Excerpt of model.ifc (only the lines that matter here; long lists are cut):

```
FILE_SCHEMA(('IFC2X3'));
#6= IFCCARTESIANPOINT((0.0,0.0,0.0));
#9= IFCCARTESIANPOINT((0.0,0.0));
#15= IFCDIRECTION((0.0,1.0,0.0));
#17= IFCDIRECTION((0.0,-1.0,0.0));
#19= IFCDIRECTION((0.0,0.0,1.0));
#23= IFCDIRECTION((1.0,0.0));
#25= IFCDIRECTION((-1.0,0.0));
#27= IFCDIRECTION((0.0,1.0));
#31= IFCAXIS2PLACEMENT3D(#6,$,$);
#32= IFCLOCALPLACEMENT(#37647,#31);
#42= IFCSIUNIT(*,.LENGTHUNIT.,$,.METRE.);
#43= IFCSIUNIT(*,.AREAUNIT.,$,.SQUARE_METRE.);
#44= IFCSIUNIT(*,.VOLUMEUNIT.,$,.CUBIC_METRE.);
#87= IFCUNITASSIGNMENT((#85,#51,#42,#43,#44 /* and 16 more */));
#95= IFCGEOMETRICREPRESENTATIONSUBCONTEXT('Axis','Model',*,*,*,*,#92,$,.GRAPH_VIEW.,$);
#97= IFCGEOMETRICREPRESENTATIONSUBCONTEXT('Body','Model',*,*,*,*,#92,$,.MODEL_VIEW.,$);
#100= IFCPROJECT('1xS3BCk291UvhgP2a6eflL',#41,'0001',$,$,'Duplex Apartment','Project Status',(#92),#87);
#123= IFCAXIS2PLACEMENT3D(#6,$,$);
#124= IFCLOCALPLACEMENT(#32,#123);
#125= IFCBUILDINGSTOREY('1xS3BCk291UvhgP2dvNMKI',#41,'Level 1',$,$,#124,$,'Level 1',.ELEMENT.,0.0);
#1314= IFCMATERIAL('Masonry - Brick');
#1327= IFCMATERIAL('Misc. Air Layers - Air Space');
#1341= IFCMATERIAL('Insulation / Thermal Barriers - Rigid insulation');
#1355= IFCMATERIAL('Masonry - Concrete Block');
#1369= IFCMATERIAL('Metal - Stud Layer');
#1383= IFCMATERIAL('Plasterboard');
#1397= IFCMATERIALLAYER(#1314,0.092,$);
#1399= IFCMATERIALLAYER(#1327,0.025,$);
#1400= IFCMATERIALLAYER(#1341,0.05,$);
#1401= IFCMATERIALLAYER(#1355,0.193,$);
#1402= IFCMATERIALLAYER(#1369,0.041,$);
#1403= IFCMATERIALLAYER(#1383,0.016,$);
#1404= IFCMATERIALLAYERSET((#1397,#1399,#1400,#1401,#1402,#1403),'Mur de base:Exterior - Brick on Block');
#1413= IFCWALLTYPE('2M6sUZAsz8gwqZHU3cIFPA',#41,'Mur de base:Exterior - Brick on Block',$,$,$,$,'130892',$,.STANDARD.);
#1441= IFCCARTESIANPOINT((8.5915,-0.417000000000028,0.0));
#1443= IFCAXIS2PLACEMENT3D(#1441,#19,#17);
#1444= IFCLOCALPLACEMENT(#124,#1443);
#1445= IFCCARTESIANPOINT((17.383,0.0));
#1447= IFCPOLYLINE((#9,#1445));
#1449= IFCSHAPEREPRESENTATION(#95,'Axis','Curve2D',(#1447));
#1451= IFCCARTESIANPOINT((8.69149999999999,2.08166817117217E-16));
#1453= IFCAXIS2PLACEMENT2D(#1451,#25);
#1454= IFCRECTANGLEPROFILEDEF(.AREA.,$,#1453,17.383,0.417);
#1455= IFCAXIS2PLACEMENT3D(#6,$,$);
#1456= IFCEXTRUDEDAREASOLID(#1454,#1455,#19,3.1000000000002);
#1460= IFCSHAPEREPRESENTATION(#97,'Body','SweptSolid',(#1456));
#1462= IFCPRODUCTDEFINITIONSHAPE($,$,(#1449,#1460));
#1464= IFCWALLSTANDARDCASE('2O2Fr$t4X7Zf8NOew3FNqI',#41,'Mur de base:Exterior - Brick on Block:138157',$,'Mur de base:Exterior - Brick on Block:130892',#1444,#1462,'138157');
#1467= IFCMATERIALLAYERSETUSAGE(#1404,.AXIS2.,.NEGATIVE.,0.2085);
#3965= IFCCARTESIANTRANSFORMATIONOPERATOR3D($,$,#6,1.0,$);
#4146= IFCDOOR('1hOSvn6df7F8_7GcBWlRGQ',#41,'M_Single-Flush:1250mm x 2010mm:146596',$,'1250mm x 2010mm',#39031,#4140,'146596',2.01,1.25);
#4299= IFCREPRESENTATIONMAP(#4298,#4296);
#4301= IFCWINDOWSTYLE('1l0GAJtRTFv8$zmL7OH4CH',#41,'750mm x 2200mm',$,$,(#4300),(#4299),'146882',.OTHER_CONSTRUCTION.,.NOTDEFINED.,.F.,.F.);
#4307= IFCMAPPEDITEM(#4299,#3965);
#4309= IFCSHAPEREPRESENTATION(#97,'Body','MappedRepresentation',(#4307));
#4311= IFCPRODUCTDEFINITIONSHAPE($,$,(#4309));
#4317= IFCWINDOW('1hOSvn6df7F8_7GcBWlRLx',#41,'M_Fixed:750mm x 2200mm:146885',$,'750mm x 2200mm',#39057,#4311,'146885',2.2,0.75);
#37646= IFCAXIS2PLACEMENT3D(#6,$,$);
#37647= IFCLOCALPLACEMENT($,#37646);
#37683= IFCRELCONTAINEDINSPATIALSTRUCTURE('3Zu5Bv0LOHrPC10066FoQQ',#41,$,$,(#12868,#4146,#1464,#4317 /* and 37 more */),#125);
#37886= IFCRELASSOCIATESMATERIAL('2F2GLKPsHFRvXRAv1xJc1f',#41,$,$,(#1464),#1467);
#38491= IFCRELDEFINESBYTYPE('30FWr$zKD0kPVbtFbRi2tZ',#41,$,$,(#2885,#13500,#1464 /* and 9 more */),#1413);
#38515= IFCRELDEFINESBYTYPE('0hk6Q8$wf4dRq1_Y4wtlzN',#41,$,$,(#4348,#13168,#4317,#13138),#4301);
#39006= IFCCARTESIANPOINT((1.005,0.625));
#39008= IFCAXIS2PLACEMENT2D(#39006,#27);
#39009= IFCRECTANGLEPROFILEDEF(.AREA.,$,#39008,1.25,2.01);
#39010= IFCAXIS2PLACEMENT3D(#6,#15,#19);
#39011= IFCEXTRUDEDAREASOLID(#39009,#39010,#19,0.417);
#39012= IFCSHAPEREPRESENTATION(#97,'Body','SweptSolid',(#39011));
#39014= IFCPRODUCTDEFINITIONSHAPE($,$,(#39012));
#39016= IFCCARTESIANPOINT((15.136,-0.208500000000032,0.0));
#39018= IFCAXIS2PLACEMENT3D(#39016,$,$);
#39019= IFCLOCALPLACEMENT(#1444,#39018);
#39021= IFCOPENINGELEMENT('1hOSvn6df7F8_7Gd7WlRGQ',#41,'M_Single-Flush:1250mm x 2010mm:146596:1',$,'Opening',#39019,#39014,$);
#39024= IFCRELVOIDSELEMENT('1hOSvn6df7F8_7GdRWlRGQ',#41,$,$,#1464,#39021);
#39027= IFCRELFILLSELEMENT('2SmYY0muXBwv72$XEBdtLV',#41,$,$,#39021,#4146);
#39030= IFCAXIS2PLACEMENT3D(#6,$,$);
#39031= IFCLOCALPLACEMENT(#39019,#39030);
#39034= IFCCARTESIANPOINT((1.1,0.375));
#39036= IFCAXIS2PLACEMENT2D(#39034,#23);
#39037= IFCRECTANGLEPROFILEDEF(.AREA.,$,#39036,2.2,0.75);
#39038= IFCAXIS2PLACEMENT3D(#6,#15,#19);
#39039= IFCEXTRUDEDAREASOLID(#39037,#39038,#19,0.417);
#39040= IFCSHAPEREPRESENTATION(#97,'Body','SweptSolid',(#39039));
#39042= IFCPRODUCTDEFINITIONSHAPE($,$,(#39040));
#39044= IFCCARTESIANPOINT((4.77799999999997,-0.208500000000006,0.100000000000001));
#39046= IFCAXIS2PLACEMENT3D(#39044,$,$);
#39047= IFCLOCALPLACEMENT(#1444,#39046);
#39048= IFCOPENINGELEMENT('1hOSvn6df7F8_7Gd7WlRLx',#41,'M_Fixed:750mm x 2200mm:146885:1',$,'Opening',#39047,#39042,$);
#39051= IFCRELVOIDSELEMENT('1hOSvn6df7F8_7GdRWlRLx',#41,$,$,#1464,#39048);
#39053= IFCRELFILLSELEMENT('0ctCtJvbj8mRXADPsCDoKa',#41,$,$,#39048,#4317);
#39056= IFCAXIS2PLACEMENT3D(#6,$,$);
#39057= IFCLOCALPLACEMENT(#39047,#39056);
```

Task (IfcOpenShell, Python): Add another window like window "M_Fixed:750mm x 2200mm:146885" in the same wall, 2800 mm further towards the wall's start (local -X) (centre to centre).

```python
import ifcopenshell
import ifcopenshell.api.feature
import ifcopenshell.api.geometry
import ifcopenshell.api.root
import ifcopenshell.geom
import ifcopenshell.util.element
import ifcopenshell.util.placement
import ifcopenshell.util.shape
import ifcopenshell.util.unit

model = ifcopenshell.open("model.ifc")
unit_scale = ifcopenshell.util.unit.calculate_unit_scale(model)
settings = ifcopenshell.geom.settings()


def volume(element):
    """Net volume in cubic metres, openings subtracted."""
    shape = ifcopenshell.geom.create_shape(settings, element)
    return ifcopenshell.util.shape.get_volume(shape.geometry)


def reuse_history(source, copy):
    """copy_class also copies each property set's owner history, people and application; keep the originals."""
    for rel in copy.IsDefinedBy:
        if rel.is_a("IfcRelDefinesByProperties") and (history := rel.RelatingPropertyDefinition.OwnerHistory):
            rel.RelatingPropertyDefinition.OwnerHistory = source.OwnerHistory
            ifcopenshell.util.element.remove_deep2(model, history)


window = model.by_guid("1hOSvn6df7F8_7GcBWlRLx")
opening = window.FillsVoids[0].RelatingOpeningElement
wall = opening.VoidsElements[0].RelatingBuildingElement
before = volume(wall)
shift = ifcopenshell.util.placement.get_local_placement(wall.ObjectPlacement)[:3, 0] * -2.8 / unit_scale

# copy_class copies the void relationship, type, container and properties, but no geometry.
new_opening = ifcopenshell.api.root.copy_class(model, product=opening)
new_opening.Representation = ifcopenshell.util.element.copy_deep(
    model, opening.Representation, exclude=["IfcGeometricRepresentationContext", "IfcRepresentationMap"]
)
new_opening.Name = "M_Fixed:750mm x 2200mm"
new_window = ifcopenshell.api.root.copy_class(model, product=window)
new_window.Representation = ifcopenshell.util.element.copy_deep(
    model, window.Representation, exclude=["IfcGeometricRepresentationContext", "IfcRepresentationMap"]
)
new_window.Name = "M_Fixed:750mm x 2200mm"
new_window.Tag = None
reuse_history(window, new_window)
fills = ifcopenshell.api.feature.add_filling(model, opening=new_opening, element=new_window)
fills.OwnerHistory = new_window.OwnerHistory  # required in IFC2X3

for old, new in ((opening, new_opening), (window, new_window)):
    matrix = ifcopenshell.util.placement.get_local_placement(old.ObjectPlacement)
    matrix[:3, 3] += shift
    ifcopenshell.api.geometry.edit_object_placement(model, product=new, matrix=matrix, is_si=False)

after = volume(wall)

print(f"wall volume {before:.3f} -> {after:.3f} m3")

model.write("model_updated.ifc")
```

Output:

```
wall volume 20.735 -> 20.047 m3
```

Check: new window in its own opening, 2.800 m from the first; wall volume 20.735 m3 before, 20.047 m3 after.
